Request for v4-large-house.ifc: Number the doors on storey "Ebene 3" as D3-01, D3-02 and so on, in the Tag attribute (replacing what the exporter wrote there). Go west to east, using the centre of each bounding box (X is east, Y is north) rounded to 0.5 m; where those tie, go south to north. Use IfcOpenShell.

First a look at what the model holds.

```python
import ifcopenshell
import ifcopenshell.util.element
import ifcopenshell.util.placement

model = ifcopenshell.open("v4-large-house.ifc")
print(model.schema)
storey = next(s for s in model.by_type("IfcBuildingStorey") if s.Name == "Ebene 3")
doors = [e for e in ifcopenshell.util.element.get_decomposition(storey) if e.is_a("IfcDoor")]
for e in sorted(doors, key=lambda e: e.id()):
    origin = ifcopenshell.util.placement.get_local_placement(e.ObjectPlacement)[:3, 3]
    print(e.id(), e.Tag, e.Name, origin.round(2) + 0.0, sep=" | ")
```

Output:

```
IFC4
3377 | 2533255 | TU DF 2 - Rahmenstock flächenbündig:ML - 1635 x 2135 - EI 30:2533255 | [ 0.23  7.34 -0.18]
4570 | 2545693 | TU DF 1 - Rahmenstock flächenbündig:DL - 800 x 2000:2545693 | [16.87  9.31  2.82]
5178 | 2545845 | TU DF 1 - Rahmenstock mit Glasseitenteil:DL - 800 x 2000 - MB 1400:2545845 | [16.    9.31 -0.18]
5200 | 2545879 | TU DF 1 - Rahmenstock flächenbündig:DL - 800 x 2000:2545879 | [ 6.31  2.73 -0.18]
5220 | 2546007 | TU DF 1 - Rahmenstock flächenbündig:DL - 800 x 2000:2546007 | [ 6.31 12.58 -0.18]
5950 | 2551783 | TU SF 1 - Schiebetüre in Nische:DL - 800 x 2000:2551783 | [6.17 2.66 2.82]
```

```python
import ifcopenshell
import ifcopenshell.geom
import ifcopenshell.util.element
import ifcopenshell.util.shape

model = ifcopenshell.open("v4-large-house.ifc")
settings = ifcopenshell.geom.settings()
settings.set("use-world-coords", True)


def centre(element):
    shape = ifcopenshell.geom.create_shape(settings, element)
    return ifcopenshell.util.shape.get_bbox_centroid(shape.geometry)


storey = next(s for s in model.by_type("IfcBuildingStorey") if s.Name == "Ebene 3")
doors = [e for e in ifcopenshell.util.element.get_decomposition(storey) if e.is_a("IfcDoor")]

# Insertion points can sit at a corner or the storey origin, so sort by the geometry (in metres).
centres = {e: centre(e) for e in doors}
doors.sort(key=lambda e: (round(centres[e][0] / 0.5), centres[e][1]))

for i, e in enumerate(doors, start=1):
    number = f"D3-{i:02d}"
    e.Tag = number
    print(e.id(), number)

model.write("v4-large-house_updated.ifc")
```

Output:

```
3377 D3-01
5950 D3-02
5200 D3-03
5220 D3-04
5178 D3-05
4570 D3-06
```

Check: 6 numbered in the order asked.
